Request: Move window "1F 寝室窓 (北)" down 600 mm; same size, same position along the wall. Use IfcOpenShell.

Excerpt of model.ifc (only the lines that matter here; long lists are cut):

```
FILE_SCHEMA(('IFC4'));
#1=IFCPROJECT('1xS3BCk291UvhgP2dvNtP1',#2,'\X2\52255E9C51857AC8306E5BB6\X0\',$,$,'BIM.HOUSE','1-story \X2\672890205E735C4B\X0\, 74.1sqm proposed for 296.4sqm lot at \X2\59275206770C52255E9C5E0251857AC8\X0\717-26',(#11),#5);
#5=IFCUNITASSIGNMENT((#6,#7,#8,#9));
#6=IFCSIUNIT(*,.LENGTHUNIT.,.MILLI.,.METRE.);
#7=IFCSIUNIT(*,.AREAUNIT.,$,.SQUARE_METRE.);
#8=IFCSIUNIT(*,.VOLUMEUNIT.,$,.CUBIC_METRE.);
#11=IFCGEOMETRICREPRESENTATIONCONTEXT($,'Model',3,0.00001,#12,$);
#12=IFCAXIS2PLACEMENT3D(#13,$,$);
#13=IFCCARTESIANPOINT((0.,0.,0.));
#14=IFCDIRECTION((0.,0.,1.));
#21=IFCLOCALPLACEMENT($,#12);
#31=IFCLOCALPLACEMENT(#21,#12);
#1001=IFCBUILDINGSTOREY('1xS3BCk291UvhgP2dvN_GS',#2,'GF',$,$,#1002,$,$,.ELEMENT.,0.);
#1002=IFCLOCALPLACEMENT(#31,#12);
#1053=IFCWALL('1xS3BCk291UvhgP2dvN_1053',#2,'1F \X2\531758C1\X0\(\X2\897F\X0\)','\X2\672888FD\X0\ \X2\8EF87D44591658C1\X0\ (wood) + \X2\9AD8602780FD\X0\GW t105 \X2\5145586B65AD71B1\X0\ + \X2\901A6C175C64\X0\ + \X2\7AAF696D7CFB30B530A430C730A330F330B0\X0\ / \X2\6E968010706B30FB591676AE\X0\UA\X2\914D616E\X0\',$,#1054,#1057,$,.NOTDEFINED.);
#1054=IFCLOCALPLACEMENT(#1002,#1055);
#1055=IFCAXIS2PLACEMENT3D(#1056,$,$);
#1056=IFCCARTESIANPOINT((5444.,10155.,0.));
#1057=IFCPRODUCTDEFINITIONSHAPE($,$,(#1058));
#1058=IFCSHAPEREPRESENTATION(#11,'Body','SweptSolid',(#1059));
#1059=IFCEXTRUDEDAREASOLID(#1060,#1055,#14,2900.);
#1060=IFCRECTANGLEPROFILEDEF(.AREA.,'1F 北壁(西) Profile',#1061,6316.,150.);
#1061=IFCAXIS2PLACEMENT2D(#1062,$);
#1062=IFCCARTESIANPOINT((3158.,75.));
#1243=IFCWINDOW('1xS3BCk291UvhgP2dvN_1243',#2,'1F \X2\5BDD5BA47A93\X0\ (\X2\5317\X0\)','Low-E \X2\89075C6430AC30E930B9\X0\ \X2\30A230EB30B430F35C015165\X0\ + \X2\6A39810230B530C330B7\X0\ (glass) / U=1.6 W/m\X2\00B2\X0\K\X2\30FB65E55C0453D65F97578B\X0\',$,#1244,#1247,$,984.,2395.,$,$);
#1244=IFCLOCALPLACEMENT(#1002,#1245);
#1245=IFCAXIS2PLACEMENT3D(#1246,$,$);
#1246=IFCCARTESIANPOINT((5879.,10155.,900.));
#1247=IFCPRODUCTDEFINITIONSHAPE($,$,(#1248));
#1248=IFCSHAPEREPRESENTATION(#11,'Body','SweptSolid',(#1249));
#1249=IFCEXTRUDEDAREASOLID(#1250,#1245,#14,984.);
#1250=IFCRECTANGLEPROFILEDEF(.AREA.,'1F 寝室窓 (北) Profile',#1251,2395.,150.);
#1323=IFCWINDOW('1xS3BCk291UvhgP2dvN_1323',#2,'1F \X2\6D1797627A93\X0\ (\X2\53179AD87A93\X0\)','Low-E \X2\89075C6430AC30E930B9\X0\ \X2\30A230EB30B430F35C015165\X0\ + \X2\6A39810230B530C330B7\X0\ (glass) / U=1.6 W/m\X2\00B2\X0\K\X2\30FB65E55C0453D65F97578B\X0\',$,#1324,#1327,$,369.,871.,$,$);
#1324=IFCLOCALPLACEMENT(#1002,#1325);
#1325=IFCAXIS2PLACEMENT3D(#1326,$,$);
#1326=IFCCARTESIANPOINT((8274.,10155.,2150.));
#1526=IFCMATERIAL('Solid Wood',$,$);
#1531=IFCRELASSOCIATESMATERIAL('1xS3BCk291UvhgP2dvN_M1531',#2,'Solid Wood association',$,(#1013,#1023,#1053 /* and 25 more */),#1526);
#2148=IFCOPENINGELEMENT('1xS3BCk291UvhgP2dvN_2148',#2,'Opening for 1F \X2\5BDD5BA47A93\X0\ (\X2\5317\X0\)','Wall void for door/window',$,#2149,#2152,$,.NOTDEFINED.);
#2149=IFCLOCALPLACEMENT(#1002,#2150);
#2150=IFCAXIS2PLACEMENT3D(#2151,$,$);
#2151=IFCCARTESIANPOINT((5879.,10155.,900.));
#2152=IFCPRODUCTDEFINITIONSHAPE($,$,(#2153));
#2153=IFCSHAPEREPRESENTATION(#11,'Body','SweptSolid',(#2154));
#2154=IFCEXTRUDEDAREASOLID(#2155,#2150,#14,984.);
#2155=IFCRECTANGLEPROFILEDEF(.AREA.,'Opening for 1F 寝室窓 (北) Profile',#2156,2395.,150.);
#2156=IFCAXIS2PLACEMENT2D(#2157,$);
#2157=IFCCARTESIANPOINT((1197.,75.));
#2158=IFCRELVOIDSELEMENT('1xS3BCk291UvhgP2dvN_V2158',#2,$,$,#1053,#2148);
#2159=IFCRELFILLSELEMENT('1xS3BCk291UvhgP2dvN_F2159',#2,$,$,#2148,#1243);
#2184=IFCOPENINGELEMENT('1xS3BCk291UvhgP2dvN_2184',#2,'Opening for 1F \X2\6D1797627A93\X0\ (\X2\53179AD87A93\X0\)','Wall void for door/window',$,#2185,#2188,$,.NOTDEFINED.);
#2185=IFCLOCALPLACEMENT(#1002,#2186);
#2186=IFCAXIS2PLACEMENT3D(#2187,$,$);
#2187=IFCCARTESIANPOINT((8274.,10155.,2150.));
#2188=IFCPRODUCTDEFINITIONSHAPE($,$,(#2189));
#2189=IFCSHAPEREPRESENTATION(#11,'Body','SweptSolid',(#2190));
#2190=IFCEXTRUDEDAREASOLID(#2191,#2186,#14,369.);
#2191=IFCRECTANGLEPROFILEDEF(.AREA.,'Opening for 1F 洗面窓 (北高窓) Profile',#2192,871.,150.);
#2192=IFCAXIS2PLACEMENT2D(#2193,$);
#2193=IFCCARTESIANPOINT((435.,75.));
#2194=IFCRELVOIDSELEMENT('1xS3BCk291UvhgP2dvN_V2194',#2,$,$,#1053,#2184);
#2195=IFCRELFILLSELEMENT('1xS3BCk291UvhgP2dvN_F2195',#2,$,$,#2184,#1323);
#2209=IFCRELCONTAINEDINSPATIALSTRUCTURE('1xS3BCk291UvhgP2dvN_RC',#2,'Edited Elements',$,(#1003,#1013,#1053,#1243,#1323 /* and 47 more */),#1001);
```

```python
import numpy as np
import ifcopenshell
import ifcopenshell.api.geometry
import ifcopenshell.util.placement
import ifcopenshell.util.unit

model = ifcopenshell.open("model.ifc")
unit_scale = ifcopenshell.util.unit.calculate_unit_scale(model)

window = model.by_guid("1xS3BCk291UvhgP2dvN_1243")
opening = window.FillsVoids[0].RelatingOpeningElement
dz = -600.0

shift = np.array([0.0, 0.0, dz])
# The window is not placed relative to its opening, so move both.
for product in (opening, window):
    matrix = ifcopenshell.util.placement.get_local_placement(product.ObjectPlacement)
    matrix[:3, 3] += shift
    ifcopenshell.api.geometry.edit_object_placement(model, product=product, matrix=matrix, is_si=False)

print(f"moved by {dz * unit_scale:+.3f} m")

model.write("model_updated.ifc")
```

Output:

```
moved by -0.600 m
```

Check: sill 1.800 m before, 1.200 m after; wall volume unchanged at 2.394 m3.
